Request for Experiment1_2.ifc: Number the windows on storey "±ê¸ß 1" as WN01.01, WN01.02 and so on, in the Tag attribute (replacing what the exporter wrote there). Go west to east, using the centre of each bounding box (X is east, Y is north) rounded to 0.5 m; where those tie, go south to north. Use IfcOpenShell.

First a look at what the model holds.

```python
import ifcopenshell
import ifcopenshell.util.element
import ifcopenshell.util.placement

model = ifcopenshell.open("Experiment1_2.ifc")
print(model.schema)
storey = next(s for s in model.by_type("IfcBuildingStorey") if s.Name == "±ê¸ß 1")
windows = [e for e in ifcopenshell.util.element.get_decomposition(storey) if e.is_a("IfcWindow")]
for e in sorted(windows, key=lambda e: e.id()):
    origin = ifcopenshell.util.placement.get_local_placement(e.ObjectPlacement)[:3, 3]
    print(e.id(), e.Tag, e.Name, origin.round(2) + 0.0, sep=" | ")
```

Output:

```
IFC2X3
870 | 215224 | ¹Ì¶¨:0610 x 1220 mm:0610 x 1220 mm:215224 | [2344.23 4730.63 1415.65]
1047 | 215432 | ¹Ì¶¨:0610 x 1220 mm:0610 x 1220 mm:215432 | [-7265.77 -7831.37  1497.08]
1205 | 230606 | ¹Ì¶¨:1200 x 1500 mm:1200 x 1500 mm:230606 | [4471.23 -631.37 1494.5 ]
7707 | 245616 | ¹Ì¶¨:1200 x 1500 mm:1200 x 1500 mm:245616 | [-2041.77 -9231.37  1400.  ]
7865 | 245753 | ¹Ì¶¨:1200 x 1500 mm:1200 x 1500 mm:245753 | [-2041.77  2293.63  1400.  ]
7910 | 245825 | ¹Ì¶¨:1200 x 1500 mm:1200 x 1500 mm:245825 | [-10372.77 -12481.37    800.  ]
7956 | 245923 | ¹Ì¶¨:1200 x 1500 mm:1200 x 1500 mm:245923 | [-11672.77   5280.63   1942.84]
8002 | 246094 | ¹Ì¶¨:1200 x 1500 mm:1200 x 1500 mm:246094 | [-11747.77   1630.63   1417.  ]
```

```python
import ifcopenshell
import ifcopenshell.geom
import ifcopenshell.util.element
import ifcopenshell.util.shape

model = ifcopenshell.open("Experiment1_2.ifc")
settings = ifcopenshell.geom.settings()
settings.set("use-world-coords", True)


def centre(element):
    shape = ifcopenshell.geom.create_shape(settings, element)
    return ifcopenshell.util.shape.get_bbox_centroid(shape.geometry)


storey = next(s for s in model.by_type("IfcBuildingStorey") if s.Name == "±ê¸ß 1")
windows = [e for e in ifcopenshell.util.element.get_decomposition(storey) if e.is_a("IfcWindow")]

# Insertion points can sit at a corner or the storey origin, so sort by the geometry (in metres).
centres = {e: centre(e) for e in windows}
windows.sort(key=lambda e: (round(centres[e][0] / 0.5), centres[e][1]))

for i, e in enumerate(windows, start=1):
    number = f"WN01.{i:02d}"
    e.Tag = number
    print(e.id(), number)

model.write("Experiment1_2_updated.ifc")
```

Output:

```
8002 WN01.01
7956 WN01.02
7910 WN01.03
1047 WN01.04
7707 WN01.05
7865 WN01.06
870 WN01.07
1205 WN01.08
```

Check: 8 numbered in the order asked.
